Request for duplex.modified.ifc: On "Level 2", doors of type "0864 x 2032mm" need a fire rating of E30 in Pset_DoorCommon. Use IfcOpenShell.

First a look at what the model holds.

```python
import ifcopenshell
import ifcopenshell.util.element

model = ifcopenshell.open("duplex.modified.ifc")
print(model.schema)
storey = next(s for s in model.by_type("IfcBuildingStorey") if s.Name == "Level 2")
doors = [e for e in ifcopenshell.util.element.get_decomposition(storey) if e.is_a("IfcDoor")]
seen = {}
for e in doors:
    element_type = ifcopenshell.util.element.get_type(e)
    key = (element_type.Name if element_type != e and element_type else None, ifcopenshell.util.element.get_pset(e, "Pset_DoorCommon", "FireRating"))
    seen[key] = seen.get(key, 0) + 1
for (name, value), count in sorted(seen.items(), key=str):
    print(count, "x", name, "|", value)
```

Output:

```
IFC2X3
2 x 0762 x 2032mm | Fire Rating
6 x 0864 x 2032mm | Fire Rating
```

```python
import ifcopenshell
import ifcopenshell.api.pset
import ifcopenshell.util.element

model = ifcopenshell.open("duplex.modified.ifc")

storey = next(s for s in model.by_type("IfcBuildingStorey") if s.Name == "Level 2")
doors = [e for e in ifcopenshell.util.element.get_decomposition(storey) if e.is_a("IfcDoor")]

count = 0
for e in doors:
    element_type = ifcopenshell.util.element.get_type(e)
    if element_type in (None, e) or element_type.Name != "0864 x 2032mm":
        continue
    # add_pset returns the element's existing set when there is one.
    pset = ifcopenshell.api.pset.add_pset(model, product=e, name="Pset_DoorCommon")
    ifcopenshell.api.pset.edit_pset(model, pset=pset, properties={"FireRating": "E30"})
    count += 1

print(count, "doors updated")

model.write("duplex.modified_updated.ifc")
```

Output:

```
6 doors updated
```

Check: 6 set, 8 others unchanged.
